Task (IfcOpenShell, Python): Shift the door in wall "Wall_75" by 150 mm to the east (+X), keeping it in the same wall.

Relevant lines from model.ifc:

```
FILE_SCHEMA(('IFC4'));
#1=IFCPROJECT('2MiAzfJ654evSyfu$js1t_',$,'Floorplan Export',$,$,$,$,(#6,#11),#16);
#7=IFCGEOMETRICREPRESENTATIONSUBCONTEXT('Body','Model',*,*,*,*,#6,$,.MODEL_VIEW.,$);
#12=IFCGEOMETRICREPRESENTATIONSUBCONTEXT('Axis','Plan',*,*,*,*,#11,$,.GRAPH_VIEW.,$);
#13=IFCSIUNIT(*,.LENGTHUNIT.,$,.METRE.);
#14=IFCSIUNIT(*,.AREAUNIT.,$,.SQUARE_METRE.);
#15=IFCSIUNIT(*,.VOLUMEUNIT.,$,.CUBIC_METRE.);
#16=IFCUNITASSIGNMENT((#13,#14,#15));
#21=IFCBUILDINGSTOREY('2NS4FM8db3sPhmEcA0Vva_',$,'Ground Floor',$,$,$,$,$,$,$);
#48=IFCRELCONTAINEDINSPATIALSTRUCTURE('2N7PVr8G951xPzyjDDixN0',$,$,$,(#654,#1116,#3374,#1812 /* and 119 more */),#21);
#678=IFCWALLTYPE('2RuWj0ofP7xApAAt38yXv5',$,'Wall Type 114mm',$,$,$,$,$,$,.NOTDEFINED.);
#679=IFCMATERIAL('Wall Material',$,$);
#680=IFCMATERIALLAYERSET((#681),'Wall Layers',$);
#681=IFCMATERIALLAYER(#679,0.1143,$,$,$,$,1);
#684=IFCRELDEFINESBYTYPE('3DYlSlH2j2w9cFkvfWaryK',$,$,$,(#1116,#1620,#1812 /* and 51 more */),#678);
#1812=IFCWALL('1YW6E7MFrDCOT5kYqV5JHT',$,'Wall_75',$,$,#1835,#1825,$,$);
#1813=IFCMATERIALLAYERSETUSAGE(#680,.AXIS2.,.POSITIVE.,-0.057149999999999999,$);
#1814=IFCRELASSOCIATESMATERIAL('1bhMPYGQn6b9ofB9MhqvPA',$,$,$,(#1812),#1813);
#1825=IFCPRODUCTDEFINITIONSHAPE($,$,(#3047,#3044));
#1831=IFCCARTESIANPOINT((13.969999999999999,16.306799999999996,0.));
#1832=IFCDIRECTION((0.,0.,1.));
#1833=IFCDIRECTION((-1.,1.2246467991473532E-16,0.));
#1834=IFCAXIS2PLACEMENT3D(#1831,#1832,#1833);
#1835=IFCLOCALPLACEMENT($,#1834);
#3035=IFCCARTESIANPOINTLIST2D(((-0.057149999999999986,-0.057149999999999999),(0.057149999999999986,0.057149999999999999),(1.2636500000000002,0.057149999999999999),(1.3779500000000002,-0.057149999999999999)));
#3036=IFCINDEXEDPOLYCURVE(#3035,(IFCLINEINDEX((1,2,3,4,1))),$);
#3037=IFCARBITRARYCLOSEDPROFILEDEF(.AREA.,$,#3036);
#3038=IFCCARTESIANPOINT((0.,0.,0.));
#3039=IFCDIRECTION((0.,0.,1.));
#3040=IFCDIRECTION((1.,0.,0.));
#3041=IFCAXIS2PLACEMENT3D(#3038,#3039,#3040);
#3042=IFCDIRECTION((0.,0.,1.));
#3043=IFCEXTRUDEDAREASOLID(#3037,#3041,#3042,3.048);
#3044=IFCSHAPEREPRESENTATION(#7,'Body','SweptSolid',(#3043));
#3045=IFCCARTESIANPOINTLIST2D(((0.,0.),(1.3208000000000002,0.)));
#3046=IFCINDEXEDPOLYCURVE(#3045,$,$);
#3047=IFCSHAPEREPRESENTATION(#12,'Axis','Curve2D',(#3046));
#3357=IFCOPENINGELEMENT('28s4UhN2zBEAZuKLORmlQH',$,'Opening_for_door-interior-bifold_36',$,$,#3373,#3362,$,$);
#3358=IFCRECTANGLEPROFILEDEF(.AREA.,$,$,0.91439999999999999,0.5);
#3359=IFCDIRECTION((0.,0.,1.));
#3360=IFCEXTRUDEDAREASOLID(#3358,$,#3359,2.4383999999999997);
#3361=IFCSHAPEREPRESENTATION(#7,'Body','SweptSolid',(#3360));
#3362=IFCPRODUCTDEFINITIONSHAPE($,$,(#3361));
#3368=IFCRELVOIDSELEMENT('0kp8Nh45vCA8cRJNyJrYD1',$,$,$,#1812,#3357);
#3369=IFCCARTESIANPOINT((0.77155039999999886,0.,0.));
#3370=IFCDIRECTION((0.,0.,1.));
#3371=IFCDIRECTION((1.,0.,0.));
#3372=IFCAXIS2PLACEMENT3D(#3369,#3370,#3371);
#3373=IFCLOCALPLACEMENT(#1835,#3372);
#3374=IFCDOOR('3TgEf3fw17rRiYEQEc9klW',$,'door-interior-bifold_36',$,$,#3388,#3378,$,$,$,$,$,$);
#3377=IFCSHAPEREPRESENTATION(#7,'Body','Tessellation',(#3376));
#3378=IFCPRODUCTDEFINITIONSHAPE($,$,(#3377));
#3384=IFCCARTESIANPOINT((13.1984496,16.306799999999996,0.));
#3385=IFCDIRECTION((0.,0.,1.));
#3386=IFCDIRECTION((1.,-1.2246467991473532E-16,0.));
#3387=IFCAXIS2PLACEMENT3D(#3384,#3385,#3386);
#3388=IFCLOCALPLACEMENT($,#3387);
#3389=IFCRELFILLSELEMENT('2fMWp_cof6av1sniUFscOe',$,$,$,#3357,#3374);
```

```python
import ifcopenshell
import ifcopenshell.api.geometry
import ifcopenshell.util.placement
import ifcopenshell.util.unit

model = ifcopenshell.open("model.ifc")
unit_scale = ifcopenshell.util.unit.calculate_unit_scale(model)

door = model.by_guid("3TgEf3fw17rRiYEQEc9klW")
opening = door.FillsVoids[0].RelatingOpeningElement
wall = opening.VoidsElements[0].RelatingBuildingElement

wall_matrix = ifcopenshell.util.placement.get_local_placement(wall.ObjectPlacement)
shift = wall_matrix[:3, 0] * -0.15 / unit_scale
before = ifcopenshell.util.placement.get_local_placement(door.ObjectPlacement)[:3, 3].copy()

# The door is not placed relative to its opening, so move both.
for product in (opening, door):
    matrix = ifcopenshell.util.placement.get_local_placement(product.ObjectPlacement)
    matrix[:3, 3] += shift
    ifcopenshell.api.geometry.edit_object_placement(model, product=product, matrix=matrix, is_si=False)

after = ifcopenshell.util.placement.get_local_placement(door.ObjectPlacement)[:3, 3]
print("door moved by", (after - before).round(3) + 0.0)

model.write("model_edited.ifc")
```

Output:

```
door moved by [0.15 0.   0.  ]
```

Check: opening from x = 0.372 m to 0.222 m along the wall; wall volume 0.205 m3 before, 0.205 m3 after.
